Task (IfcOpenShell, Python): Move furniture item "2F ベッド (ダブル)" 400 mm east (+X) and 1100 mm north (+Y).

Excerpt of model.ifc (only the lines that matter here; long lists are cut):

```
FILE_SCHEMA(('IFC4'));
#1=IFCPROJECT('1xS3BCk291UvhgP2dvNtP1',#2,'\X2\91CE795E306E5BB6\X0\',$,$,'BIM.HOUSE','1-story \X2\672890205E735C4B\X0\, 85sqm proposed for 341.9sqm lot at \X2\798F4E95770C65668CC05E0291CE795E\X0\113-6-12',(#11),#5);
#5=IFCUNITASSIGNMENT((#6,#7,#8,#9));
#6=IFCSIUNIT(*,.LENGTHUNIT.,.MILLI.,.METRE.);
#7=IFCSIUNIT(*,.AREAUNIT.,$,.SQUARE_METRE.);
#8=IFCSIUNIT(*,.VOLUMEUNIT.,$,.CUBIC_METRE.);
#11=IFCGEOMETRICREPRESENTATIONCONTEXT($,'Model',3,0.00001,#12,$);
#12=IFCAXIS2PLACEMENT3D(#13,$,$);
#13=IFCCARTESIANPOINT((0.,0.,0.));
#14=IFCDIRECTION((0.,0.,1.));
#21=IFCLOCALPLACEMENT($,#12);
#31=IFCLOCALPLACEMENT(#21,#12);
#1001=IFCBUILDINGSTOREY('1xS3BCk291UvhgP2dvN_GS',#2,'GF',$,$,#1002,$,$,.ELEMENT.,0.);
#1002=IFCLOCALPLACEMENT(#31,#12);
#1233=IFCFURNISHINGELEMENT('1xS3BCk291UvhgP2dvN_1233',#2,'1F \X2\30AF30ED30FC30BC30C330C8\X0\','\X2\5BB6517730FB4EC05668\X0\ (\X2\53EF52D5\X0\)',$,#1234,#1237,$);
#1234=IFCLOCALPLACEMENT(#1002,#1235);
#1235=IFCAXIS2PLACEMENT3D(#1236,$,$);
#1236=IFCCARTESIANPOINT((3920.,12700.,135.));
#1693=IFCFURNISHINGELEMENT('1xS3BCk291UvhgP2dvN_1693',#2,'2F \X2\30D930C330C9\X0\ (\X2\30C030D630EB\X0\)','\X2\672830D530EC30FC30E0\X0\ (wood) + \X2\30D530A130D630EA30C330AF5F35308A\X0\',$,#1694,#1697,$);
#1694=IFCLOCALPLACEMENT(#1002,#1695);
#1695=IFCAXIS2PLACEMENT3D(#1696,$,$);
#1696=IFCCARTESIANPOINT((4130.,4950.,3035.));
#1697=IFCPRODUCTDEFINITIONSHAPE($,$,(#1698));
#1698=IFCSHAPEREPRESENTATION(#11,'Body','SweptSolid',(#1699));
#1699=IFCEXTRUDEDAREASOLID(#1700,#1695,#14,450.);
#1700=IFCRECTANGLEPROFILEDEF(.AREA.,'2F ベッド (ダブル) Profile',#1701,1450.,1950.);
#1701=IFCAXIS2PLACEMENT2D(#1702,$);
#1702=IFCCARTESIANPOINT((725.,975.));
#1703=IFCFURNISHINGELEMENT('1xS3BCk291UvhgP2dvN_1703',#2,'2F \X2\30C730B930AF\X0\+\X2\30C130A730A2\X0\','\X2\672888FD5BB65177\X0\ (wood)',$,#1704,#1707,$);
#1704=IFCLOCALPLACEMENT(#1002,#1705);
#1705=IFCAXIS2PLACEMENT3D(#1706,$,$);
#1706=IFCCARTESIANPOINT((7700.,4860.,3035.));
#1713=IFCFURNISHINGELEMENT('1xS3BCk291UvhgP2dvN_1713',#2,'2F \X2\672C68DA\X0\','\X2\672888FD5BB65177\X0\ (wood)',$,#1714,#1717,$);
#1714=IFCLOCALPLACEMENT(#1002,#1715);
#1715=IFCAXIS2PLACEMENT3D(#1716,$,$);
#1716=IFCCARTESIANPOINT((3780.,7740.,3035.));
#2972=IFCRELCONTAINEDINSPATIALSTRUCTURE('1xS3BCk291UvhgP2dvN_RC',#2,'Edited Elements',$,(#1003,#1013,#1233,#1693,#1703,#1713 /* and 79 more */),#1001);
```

```python
import ifcopenshell
import ifcopenshell.api.geometry
import ifcopenshell.util.placement
import ifcopenshell.util.unit

model = ifcopenshell.open("model.ifc")
unit_scale = ifcopenshell.util.unit.calculate_unit_scale(model)

item = model.by_guid("1xS3BCk291UvhgP2dvN_1693")
matrix = ifcopenshell.util.placement.get_local_placement(item.ObjectPlacement)
matrix[0, 3] += 0.4 / unit_scale
matrix[1, 3] += 1.1 / unit_scale
ifcopenshell.api.geometry.edit_object_placement(model, product=item, matrix=matrix, is_si=False)

print(ifcopenshell.util.placement.get_local_placement(item.ObjectPlacement).round(3) + 0.0)

model.write("model_edited.ifc")
```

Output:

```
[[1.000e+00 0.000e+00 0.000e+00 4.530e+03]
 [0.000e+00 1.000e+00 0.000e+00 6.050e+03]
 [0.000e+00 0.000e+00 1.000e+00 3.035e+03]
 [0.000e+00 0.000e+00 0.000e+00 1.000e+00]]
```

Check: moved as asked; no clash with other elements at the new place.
